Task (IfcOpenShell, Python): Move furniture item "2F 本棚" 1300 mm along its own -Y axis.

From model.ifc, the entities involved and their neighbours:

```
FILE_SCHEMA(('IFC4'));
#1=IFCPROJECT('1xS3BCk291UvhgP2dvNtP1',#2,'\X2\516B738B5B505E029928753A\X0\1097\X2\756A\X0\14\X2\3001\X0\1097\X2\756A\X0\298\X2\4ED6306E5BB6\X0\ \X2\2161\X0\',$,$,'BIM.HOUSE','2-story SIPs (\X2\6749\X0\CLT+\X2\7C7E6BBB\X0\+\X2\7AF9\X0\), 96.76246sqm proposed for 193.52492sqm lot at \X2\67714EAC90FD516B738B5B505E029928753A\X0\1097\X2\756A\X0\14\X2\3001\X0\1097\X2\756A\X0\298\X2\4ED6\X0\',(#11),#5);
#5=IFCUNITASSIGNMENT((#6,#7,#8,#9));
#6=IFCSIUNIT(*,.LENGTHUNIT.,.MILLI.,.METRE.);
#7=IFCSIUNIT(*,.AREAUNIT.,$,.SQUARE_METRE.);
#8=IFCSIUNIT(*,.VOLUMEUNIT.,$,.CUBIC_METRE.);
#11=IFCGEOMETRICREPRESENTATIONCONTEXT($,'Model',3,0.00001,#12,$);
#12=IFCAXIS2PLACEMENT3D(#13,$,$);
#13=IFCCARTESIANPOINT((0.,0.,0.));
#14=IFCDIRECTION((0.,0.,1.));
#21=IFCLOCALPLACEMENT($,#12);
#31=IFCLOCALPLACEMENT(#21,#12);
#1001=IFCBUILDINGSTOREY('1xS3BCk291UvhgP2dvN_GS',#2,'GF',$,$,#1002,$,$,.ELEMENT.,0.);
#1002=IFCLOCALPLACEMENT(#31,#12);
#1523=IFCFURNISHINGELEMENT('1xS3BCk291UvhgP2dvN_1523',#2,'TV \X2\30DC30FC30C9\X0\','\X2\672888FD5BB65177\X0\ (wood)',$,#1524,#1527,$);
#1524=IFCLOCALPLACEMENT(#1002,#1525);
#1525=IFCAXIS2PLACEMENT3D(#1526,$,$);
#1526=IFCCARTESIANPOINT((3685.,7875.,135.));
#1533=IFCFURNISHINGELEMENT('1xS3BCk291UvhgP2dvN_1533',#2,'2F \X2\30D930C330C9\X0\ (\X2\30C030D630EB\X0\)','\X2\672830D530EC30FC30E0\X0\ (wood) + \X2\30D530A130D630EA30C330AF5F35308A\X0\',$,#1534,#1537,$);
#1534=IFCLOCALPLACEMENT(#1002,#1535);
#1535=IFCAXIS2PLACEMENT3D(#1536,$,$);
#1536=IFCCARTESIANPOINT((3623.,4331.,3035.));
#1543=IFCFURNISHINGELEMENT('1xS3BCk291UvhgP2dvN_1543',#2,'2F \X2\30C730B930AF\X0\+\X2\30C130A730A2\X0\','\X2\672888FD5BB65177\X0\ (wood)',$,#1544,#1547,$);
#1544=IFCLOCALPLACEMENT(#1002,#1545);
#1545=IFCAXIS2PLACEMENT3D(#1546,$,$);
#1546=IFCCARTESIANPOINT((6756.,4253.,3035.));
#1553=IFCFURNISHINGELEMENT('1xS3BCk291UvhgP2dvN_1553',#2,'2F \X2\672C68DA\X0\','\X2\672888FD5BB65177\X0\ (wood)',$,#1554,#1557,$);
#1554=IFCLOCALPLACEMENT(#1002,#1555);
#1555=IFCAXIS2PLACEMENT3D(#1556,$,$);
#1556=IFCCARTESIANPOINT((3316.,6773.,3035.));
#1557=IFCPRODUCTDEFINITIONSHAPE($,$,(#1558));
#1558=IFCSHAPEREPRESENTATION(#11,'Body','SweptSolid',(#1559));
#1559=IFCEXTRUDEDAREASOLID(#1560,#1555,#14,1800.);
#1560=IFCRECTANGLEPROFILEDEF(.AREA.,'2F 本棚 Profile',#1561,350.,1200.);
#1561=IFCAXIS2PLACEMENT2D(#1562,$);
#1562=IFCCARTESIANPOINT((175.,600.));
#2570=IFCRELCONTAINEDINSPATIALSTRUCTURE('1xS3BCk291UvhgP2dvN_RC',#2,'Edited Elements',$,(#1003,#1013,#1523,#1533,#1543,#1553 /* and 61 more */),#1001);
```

```python
import ifcopenshell
import ifcopenshell.api.geometry
import ifcopenshell.util.placement
import ifcopenshell.util.unit

model = ifcopenshell.open("model.ifc")
unit_scale = ifcopenshell.util.unit.calculate_unit_scale(model)

item = model.by_guid("1xS3BCk291UvhgP2dvN_1553")
matrix = ifcopenshell.util.placement.get_local_placement(item.ObjectPlacement)
matrix[:3, 3] -= matrix[:3, 1] * 1.3 / unit_scale
ifcopenshell.api.geometry.edit_object_placement(model, product=item, matrix=matrix, is_si=False)

print(ifcopenshell.util.placement.get_local_placement(item.ObjectPlacement).round(3) + 0.0)

model.write("model_rev.ifc")
```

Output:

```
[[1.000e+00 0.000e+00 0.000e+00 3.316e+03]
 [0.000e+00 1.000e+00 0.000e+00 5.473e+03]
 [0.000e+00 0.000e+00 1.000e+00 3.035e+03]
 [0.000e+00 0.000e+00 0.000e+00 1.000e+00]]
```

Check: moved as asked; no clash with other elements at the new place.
